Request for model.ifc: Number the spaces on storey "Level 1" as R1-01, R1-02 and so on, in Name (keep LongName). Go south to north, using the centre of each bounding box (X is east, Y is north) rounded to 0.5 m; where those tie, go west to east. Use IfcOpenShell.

First a look at what the model holds.

```python
import ifcopenshell
import ifcopenshell.util.element
import ifcopenshell.util.placement

model = ifcopenshell.open("model.ifc")
print(model.schema)
storey = next(s for s in model.by_type("IfcBuildingStorey") if s.Name == "Level 1")
spaces = [e for e in ifcopenshell.util.element.get_decomposition(storey) if e.is_a("IfcSpace")]
for e in sorted(spaces, key=lambda e: e.id()):
    origin = ifcopenshell.util.placement.get_local_placement(e.ObjectPlacement)[:3, 3]
    print(e.id(), e.Name, e.LongName, origin.round(2) + 0.0, sep=" | ")
```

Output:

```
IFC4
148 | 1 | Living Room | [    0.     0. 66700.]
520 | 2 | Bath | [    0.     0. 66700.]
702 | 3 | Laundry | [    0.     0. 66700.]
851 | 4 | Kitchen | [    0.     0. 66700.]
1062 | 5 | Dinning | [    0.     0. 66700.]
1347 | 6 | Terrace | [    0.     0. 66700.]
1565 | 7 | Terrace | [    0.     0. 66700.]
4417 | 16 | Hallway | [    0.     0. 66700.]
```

```python
import ifcopenshell
import ifcopenshell.geom
import ifcopenshell.util.element
import ifcopenshell.util.shape

model = ifcopenshell.open("model.ifc")
settings = ifcopenshell.geom.settings()
settings.set("use-world-coords", True)


def centre(element):
    shape = ifcopenshell.geom.create_shape(settings, element)
    return ifcopenshell.util.shape.get_bbox_centroid(shape.geometry)


storey = next(s for s in model.by_type("IfcBuildingStorey") if s.Name == "Level 1")
spaces = [e for e in ifcopenshell.util.element.get_decomposition(storey) if e.is_a("IfcSpace")]

# Insertion points can sit at a corner or the storey origin, so sort by the geometry (in metres).
centres = {e: centre(e) for e in spaces}
spaces.sort(key=lambda e: (round(centres[e][1] / 0.5), centres[e][0]))

for i, e in enumerate(spaces, start=1):
    number = f"R1-{i:02d}"
    e.Name = number
    print(e.id(), number)

model.write("model_rev.ifc")
```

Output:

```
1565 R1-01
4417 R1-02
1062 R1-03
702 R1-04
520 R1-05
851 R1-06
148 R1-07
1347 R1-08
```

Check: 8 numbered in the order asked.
